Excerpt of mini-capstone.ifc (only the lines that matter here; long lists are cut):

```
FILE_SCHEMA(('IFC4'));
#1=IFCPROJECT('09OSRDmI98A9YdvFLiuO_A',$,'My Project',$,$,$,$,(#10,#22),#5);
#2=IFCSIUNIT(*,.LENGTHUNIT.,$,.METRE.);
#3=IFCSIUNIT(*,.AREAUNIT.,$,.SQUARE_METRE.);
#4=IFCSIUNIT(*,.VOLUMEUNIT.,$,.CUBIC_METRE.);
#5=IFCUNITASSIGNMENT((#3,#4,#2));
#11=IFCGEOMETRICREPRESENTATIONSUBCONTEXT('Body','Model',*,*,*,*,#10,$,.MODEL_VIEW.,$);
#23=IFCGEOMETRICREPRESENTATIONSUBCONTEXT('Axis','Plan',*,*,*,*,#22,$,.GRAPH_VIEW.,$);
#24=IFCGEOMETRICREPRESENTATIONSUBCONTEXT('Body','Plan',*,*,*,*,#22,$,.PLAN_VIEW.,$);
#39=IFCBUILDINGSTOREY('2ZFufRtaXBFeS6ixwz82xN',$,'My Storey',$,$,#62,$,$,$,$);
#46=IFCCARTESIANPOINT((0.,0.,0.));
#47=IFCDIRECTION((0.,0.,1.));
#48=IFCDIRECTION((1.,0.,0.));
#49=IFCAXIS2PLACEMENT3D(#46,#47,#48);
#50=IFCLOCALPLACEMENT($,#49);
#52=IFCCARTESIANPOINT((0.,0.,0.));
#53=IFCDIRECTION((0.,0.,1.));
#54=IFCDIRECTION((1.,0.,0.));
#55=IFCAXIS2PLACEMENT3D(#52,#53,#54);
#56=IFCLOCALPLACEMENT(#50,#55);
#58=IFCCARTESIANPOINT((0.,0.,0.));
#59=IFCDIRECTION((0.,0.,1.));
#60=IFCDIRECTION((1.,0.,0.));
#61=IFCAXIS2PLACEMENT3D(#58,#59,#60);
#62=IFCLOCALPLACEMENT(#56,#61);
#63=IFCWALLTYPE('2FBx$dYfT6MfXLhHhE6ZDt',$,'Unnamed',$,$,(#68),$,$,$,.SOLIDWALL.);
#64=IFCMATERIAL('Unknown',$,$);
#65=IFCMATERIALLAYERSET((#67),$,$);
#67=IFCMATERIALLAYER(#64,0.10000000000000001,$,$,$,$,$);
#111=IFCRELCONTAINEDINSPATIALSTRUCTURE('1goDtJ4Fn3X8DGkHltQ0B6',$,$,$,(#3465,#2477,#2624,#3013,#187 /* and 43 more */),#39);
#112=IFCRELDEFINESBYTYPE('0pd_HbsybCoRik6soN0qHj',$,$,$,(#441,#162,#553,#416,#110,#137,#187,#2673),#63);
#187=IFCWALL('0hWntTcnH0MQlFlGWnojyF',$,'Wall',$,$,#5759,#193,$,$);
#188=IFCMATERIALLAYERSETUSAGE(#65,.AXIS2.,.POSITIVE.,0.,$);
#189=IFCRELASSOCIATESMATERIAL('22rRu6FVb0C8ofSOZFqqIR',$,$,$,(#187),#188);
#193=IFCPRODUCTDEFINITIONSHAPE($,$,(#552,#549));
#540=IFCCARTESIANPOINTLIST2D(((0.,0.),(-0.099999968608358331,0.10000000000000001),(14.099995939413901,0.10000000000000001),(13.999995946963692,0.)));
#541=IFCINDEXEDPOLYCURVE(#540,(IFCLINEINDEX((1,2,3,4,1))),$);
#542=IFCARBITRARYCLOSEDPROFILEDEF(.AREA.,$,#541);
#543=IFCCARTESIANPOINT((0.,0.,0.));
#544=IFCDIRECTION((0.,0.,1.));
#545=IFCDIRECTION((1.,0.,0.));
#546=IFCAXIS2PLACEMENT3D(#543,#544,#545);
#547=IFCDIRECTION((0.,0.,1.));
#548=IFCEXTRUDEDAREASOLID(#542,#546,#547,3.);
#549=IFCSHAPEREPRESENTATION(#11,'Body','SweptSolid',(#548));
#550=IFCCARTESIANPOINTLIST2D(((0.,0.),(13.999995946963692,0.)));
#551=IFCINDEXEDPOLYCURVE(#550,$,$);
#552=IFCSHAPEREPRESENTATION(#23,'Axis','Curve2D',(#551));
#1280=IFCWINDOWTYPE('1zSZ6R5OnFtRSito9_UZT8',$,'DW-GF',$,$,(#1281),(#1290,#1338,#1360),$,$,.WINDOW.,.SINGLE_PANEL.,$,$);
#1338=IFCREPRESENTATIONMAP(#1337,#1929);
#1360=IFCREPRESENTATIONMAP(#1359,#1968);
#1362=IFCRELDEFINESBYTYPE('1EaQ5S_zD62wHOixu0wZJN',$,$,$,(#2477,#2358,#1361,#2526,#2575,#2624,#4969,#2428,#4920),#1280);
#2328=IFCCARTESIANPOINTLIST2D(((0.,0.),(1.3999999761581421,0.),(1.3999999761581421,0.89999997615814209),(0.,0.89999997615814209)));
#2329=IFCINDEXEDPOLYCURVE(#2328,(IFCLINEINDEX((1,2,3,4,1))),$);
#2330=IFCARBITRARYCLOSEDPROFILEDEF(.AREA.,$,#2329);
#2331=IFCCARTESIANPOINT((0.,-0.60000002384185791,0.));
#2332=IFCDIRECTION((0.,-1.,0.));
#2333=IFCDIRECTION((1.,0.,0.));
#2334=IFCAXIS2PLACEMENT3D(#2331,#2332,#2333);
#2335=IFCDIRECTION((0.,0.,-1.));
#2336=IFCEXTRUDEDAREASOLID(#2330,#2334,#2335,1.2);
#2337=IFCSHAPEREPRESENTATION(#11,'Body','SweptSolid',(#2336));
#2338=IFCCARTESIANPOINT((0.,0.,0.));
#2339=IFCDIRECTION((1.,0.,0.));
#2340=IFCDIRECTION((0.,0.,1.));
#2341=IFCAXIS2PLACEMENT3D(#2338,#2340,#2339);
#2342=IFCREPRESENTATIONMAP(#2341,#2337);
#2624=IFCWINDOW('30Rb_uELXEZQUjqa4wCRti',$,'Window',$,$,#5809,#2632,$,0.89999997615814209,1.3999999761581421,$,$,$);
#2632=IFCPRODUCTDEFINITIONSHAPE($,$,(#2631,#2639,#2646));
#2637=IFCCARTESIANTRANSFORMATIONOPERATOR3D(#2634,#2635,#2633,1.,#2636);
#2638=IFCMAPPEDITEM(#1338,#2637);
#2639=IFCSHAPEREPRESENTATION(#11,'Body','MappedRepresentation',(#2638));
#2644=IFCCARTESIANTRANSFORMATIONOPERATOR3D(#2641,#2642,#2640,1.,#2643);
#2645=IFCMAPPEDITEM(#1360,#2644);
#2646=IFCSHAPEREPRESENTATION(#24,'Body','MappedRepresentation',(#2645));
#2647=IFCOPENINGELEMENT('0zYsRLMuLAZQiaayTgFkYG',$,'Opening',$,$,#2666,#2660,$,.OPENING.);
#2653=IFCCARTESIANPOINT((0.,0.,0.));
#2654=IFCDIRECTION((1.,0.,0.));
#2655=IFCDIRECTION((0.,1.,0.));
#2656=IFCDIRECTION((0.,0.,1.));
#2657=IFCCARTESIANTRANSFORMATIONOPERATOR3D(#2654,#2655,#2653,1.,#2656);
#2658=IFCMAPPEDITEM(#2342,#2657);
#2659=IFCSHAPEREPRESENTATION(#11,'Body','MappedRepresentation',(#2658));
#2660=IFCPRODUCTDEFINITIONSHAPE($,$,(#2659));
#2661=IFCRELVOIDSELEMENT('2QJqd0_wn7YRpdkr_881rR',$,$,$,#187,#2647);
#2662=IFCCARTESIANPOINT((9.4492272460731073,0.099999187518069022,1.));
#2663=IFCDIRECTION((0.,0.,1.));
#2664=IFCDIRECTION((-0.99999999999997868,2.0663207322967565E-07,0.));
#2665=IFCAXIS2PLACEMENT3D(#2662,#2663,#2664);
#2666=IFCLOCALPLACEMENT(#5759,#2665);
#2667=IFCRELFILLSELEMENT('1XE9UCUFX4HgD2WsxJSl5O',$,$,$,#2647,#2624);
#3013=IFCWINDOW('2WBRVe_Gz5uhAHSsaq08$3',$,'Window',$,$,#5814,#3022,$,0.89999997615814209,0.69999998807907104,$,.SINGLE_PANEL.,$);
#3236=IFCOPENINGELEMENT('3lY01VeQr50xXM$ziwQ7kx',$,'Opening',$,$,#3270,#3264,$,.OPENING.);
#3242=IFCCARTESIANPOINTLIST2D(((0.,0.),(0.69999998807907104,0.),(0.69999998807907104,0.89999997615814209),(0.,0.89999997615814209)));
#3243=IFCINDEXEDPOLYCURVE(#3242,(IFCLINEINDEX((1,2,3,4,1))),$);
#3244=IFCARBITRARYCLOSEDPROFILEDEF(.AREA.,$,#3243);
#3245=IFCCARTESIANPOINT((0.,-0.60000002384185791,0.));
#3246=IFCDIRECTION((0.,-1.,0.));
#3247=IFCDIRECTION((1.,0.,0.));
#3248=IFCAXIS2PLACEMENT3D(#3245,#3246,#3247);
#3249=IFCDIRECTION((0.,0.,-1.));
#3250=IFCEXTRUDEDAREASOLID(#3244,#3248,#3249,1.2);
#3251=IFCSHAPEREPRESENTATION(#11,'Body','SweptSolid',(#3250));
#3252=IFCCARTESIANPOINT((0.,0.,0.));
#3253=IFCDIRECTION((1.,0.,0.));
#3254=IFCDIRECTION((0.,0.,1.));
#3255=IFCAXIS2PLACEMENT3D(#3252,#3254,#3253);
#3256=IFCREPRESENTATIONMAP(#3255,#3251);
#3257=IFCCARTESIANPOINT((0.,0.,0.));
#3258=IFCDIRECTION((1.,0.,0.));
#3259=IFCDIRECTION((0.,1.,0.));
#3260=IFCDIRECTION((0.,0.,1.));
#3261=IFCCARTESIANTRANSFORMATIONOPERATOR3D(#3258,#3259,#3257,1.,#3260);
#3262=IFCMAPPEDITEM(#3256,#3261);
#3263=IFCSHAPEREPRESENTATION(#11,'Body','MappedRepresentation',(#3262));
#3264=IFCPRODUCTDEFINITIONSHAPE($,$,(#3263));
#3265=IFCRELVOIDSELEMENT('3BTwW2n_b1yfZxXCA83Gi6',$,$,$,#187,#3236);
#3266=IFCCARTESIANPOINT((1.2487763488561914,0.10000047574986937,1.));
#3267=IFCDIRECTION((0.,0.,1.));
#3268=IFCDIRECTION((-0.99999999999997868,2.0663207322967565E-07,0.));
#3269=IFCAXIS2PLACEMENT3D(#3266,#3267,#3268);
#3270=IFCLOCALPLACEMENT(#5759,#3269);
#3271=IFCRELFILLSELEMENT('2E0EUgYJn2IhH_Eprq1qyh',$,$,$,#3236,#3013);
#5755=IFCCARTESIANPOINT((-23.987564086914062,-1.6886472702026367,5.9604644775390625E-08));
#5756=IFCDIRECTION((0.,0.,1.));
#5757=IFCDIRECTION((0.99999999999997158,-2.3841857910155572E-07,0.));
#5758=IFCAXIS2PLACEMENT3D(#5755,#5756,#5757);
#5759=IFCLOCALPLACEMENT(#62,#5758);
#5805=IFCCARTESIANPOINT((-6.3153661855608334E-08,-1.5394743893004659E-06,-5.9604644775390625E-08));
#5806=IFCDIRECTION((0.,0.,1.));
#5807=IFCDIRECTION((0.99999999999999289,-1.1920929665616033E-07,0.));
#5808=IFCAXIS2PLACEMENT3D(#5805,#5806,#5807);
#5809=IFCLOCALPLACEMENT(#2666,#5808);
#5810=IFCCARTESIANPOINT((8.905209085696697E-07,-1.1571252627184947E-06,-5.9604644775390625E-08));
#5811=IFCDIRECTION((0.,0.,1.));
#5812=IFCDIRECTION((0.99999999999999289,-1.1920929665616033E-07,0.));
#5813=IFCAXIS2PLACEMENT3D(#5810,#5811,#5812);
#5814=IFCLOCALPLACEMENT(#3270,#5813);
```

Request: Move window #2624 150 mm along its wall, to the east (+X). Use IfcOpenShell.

```python
import ifcopenshell
import ifcopenshell.api.geometry
import ifcopenshell.util.placement
import ifcopenshell.util.unit

model = ifcopenshell.open("mini-capstone.ifc")
unit_scale = ifcopenshell.util.unit.calculate_unit_scale(model)

window = model.by_guid("30Rb_uELXEZQUjqa4wCRti")
opening = window.FillsVoids[0].RelatingOpeningElement
wall = opening.VoidsElements[0].RelatingBuildingElement

wall_matrix = ifcopenshell.util.placement.get_local_placement(wall.ObjectPlacement)
shift = wall_matrix[:3, 0] * 0.15 / unit_scale
before = ifcopenshell.util.placement.get_local_placement(window.ObjectPlacement)[:3, 3].copy()

# The window is placed relative to its opening, so it follows when the opening moves.
matrix = ifcopenshell.util.placement.get_local_placement(opening.ObjectPlacement)
matrix[:3, 3] += shift
ifcopenshell.api.geometry.edit_object_placement(
    model, product=opening, matrix=matrix, is_si=False, should_transform_children=True
)

after = ifcopenshell.util.placement.get_local_placement(window.ObjectPlacement)[:3, 3]
print("window moved by", (after - before).round(3) + 0.0)

model.write("mini-capstone_v2.ifc")
```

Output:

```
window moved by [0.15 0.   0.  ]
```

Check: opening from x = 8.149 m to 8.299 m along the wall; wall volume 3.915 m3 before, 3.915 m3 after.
